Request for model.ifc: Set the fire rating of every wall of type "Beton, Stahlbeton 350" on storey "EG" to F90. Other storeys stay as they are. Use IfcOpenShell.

First a look at what the model holds.

```python
import ifcopenshell
import ifcopenshell.util.element

model = ifcopenshell.open("model.ifc")
print(model.schema)
storey = next(s for s in model.by_type("IfcBuildingStorey") if s.Name == "EG")
walls = [e for e in ifcopenshell.util.element.get_decomposition(storey) if e.is_a("IfcWall")]
seen = {}
for e in walls:
    element_type = ifcopenshell.util.element.get_type(e)
    key = (element_type.Name if element_type != e and element_type else None, ifcopenshell.util.element.get_pset(e, "Pset_WallCommon", "FireRating"))
    seen[key] = seen.get(key, 0) + 1
for (name, value), count in sorted(seen.items(), key=str):
    print(count, "x", name, "|", value)
```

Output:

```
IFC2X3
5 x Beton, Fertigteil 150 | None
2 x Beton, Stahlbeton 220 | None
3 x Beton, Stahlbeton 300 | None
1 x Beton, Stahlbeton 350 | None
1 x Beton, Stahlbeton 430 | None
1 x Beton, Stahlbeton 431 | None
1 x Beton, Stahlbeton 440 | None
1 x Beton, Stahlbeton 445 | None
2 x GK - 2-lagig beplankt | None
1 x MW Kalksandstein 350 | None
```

```python
import ifcopenshell
import ifcopenshell.api.pset
import ifcopenshell.util.element

model = ifcopenshell.open("model.ifc")

storey = next(s for s in model.by_type("IfcBuildingStorey") if s.Name == "EG")
walls = [e for e in ifcopenshell.util.element.get_decomposition(storey) if e.is_a("IfcWall")]

count = 0
for e in walls:
    element_type = ifcopenshell.util.element.get_type(e)
    if element_type in (None, e) or element_type.Name != "Beton, Stahlbeton 350":
        continue
    # add_pset returns the element's existing set when there is one.
    pset = ifcopenshell.api.pset.add_pset(model, product=e, name="Pset_WallCommon")
    ifcopenshell.api.pset.edit_pset(model, pset=pset, properties={"FireRating": "F90"})
    count += 1

print(count, "walls updated")

model.write("model_rev.ifc")
```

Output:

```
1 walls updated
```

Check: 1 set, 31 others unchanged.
